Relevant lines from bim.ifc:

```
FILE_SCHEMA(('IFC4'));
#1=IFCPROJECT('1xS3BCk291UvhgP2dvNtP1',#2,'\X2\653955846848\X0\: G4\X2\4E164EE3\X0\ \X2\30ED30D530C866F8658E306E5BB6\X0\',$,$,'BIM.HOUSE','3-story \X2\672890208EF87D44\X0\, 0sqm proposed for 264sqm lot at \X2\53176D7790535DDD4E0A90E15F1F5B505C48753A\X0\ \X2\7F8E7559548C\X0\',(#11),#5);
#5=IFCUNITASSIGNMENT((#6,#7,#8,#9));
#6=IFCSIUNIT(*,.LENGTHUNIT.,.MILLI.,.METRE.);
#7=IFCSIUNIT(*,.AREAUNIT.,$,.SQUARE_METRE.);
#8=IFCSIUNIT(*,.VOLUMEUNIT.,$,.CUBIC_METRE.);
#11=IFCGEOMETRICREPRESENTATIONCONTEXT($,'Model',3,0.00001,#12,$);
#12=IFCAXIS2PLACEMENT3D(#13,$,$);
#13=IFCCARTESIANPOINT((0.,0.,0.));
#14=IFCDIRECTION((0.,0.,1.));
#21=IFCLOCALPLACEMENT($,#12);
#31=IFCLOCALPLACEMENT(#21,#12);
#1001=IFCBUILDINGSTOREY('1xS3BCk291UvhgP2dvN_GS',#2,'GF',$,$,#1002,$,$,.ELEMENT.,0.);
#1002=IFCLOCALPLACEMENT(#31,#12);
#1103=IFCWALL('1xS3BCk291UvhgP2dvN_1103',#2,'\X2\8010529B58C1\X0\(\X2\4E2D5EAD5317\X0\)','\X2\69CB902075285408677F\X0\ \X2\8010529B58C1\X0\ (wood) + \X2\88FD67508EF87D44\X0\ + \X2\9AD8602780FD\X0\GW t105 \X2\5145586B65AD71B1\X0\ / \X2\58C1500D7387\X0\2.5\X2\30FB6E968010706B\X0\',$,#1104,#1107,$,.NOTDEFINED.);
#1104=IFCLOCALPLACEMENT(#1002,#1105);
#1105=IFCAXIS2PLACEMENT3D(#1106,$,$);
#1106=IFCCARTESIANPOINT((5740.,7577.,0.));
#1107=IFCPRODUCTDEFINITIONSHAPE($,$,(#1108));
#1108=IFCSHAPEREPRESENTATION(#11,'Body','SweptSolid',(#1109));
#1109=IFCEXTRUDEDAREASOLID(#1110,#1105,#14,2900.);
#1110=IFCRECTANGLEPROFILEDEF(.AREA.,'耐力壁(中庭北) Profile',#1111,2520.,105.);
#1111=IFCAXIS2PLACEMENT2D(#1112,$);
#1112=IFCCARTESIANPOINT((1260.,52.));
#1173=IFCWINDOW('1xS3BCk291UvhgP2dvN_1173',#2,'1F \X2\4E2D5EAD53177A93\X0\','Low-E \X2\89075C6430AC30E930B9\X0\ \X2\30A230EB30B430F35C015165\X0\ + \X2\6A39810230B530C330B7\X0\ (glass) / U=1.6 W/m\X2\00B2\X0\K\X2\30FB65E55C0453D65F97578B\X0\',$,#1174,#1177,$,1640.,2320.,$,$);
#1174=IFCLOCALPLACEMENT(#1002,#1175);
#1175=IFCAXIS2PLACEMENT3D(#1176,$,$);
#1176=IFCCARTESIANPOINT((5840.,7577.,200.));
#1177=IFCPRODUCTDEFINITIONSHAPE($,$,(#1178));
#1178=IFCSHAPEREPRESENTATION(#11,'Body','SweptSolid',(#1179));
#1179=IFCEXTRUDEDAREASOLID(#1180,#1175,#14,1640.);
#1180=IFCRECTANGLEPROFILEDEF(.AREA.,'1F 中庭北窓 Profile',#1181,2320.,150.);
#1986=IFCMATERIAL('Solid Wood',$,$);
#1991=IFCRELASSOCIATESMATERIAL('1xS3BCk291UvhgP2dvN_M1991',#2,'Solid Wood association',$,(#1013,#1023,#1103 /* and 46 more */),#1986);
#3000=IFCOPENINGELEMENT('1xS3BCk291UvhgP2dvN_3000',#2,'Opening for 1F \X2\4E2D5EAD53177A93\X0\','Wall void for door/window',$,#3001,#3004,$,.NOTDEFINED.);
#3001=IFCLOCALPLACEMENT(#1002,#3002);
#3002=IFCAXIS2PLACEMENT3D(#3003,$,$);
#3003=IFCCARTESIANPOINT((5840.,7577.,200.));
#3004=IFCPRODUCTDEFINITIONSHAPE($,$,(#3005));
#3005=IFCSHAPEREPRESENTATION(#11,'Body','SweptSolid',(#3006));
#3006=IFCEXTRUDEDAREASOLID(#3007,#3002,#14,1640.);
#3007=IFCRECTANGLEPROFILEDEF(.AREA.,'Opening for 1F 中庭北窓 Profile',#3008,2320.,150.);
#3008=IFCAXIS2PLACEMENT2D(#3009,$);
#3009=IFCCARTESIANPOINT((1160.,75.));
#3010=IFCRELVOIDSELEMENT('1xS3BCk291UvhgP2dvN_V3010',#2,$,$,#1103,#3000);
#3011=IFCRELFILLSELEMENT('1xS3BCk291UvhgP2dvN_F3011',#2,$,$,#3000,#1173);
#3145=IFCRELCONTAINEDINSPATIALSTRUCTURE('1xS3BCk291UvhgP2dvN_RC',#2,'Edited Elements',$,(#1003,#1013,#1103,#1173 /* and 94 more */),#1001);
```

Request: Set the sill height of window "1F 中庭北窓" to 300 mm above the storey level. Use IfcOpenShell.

```python
import numpy as np
import ifcopenshell
import ifcopenshell.api.geometry
import ifcopenshell.geom
import ifcopenshell.util.element
import ifcopenshell.util.placement
import ifcopenshell.util.shape
import ifcopenshell.util.unit

model = ifcopenshell.open("bim.ifc")
unit_scale = ifcopenshell.util.unit.calculate_unit_scale(model)

window = model.by_guid("1xS3BCk291UvhgP2dvN_1173")
opening = window.FillsVoids[0].RelatingOpeningElement
storey = ifcopenshell.util.element.get_container(window, ifc_class="IfcBuildingStorey")
level = ifcopenshell.util.placement.get_local_placement(storey.ObjectPlacement)[2, 3]

# The opening's origin need not be at the sill, so measure its lowest point.
shape = ifcopenshell.geom.create_shape(ifcopenshell.geom.settings(), opening)
bottom = ifcopenshell.util.shape.get_shape_bottom_elevation(shape, shape.geometry) / unit_scale
dz = level + 0.3 / unit_scale - bottom

shift = np.array([0.0, 0.0, dz])
# The window is not placed relative to its opening, so move both.
for product in (opening, window):
    matrix = ifcopenshell.util.placement.get_local_placement(product.ObjectPlacement)
    matrix[:3, 3] += shift
    ifcopenshell.api.geometry.edit_object_placement(model, product=product, matrix=matrix, is_si=False)

print(f"moved by {dz * unit_scale:+.3f} m")

model.write("bim-out.ifc")
```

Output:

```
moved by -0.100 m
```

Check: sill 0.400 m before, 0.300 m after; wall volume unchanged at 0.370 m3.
